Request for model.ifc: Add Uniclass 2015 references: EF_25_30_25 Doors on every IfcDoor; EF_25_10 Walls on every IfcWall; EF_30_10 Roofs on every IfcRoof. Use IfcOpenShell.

First a look at what the model holds.

```python
import ifcopenshell

model = ifcopenshell.open("model.ifc")
print(model.schema)
print("classifications:", [c.Name for c in model.by_type("IfcClassification")])
for ifc_class in ("IfcDoor", "IfcRoof", "IfcStair", "IfcWall", "IfcWindow"):
    print(ifc_class, len(model.by_type(ifc_class)))
```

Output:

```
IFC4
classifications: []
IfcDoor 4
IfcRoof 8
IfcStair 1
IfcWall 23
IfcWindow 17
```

```python
import ifcopenshell
import ifcopenshell.api.classification

model = ifcopenshell.open("model.ifc")

system = ifcopenshell.api.classification.add_classification(model, classification="Uniclass 2015")

codes = {
    "IfcDoor": ("EF_25_30_25", "Doors"),
    "IfcWall": ("EF_25_10", "Walls"),
    "IfcRoof": ("EF_30_10", "Roofs"),
}
for ifc_class, (code, name) in codes.items():
    products = model.by_type(ifc_class)
    ifcopenshell.api.classification.add_reference(
        model, products=products, classification=system, identification=code, name=name
    )
    print(code, len(products))

model.write("model_edited.ifc")
```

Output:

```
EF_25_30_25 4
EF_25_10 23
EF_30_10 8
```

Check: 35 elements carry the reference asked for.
